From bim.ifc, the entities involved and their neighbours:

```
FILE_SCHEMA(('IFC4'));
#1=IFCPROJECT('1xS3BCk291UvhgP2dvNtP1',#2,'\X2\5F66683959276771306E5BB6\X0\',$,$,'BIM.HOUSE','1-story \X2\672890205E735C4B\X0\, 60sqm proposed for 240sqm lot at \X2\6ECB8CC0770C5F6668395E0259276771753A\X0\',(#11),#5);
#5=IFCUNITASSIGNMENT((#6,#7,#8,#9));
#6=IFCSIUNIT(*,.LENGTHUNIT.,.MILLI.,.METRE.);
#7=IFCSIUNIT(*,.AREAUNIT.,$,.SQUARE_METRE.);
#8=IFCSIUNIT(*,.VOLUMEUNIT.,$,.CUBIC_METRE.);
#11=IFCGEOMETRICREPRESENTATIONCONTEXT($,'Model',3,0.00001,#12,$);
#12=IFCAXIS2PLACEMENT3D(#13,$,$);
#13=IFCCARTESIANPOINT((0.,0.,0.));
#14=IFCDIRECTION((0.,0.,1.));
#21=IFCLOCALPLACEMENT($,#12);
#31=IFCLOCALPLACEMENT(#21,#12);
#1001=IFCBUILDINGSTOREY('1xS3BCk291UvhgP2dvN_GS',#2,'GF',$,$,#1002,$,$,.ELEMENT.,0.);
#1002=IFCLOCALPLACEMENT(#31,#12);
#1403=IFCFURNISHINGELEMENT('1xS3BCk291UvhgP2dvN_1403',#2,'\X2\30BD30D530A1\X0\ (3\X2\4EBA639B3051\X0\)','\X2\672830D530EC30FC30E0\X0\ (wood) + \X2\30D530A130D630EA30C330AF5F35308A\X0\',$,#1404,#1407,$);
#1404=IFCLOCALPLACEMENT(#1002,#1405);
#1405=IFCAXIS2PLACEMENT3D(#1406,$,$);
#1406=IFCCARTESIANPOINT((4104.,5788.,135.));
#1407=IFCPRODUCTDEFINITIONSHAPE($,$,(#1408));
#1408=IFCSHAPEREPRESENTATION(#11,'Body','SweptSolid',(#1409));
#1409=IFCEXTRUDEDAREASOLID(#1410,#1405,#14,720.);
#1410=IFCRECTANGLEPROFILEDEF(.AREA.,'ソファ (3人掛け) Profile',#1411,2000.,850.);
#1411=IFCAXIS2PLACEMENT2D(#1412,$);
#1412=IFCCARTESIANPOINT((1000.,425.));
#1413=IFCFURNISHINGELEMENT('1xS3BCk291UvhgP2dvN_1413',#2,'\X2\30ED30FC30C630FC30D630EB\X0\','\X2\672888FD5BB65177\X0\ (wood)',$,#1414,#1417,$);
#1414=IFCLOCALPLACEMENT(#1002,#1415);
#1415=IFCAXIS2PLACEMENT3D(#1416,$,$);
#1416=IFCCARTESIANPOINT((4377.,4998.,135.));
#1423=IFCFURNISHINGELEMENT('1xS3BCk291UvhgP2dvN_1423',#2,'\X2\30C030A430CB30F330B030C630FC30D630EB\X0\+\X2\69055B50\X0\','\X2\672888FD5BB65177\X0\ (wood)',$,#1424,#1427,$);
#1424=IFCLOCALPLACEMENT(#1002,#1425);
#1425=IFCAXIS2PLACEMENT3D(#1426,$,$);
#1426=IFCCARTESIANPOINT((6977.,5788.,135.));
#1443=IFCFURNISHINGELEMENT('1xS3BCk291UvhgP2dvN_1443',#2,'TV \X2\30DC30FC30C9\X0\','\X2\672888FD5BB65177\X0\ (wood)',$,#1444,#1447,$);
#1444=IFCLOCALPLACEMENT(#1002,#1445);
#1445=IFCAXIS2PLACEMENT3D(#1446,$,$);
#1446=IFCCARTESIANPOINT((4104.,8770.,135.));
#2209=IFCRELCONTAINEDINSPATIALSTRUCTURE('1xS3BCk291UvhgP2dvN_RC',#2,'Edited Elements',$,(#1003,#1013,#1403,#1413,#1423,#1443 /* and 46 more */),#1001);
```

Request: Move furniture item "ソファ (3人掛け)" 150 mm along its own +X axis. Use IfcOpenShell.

```python
import ifcopenshell
import ifcopenshell.api.geometry
import ifcopenshell.util.placement

model = ifcopenshell.open("bim.ifc")

item = model.by_id(1403)
matrix = ifcopenshell.util.placement.get_local_placement(item.ObjectPlacement)
matrix[:3, 3] += matrix[:3, 0] * 150.0
ifcopenshell.api.geometry.edit_object_placement(model, product=item, matrix=matrix, is_si=False)

print(ifcopenshell.util.placement.get_local_placement(item.ObjectPlacement).round(3) + 0.0)

model.write("bim_v2.ifc")
```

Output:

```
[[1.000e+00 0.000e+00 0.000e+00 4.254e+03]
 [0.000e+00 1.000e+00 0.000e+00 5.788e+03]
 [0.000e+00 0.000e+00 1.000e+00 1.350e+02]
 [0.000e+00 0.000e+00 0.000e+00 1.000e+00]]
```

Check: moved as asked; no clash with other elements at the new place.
